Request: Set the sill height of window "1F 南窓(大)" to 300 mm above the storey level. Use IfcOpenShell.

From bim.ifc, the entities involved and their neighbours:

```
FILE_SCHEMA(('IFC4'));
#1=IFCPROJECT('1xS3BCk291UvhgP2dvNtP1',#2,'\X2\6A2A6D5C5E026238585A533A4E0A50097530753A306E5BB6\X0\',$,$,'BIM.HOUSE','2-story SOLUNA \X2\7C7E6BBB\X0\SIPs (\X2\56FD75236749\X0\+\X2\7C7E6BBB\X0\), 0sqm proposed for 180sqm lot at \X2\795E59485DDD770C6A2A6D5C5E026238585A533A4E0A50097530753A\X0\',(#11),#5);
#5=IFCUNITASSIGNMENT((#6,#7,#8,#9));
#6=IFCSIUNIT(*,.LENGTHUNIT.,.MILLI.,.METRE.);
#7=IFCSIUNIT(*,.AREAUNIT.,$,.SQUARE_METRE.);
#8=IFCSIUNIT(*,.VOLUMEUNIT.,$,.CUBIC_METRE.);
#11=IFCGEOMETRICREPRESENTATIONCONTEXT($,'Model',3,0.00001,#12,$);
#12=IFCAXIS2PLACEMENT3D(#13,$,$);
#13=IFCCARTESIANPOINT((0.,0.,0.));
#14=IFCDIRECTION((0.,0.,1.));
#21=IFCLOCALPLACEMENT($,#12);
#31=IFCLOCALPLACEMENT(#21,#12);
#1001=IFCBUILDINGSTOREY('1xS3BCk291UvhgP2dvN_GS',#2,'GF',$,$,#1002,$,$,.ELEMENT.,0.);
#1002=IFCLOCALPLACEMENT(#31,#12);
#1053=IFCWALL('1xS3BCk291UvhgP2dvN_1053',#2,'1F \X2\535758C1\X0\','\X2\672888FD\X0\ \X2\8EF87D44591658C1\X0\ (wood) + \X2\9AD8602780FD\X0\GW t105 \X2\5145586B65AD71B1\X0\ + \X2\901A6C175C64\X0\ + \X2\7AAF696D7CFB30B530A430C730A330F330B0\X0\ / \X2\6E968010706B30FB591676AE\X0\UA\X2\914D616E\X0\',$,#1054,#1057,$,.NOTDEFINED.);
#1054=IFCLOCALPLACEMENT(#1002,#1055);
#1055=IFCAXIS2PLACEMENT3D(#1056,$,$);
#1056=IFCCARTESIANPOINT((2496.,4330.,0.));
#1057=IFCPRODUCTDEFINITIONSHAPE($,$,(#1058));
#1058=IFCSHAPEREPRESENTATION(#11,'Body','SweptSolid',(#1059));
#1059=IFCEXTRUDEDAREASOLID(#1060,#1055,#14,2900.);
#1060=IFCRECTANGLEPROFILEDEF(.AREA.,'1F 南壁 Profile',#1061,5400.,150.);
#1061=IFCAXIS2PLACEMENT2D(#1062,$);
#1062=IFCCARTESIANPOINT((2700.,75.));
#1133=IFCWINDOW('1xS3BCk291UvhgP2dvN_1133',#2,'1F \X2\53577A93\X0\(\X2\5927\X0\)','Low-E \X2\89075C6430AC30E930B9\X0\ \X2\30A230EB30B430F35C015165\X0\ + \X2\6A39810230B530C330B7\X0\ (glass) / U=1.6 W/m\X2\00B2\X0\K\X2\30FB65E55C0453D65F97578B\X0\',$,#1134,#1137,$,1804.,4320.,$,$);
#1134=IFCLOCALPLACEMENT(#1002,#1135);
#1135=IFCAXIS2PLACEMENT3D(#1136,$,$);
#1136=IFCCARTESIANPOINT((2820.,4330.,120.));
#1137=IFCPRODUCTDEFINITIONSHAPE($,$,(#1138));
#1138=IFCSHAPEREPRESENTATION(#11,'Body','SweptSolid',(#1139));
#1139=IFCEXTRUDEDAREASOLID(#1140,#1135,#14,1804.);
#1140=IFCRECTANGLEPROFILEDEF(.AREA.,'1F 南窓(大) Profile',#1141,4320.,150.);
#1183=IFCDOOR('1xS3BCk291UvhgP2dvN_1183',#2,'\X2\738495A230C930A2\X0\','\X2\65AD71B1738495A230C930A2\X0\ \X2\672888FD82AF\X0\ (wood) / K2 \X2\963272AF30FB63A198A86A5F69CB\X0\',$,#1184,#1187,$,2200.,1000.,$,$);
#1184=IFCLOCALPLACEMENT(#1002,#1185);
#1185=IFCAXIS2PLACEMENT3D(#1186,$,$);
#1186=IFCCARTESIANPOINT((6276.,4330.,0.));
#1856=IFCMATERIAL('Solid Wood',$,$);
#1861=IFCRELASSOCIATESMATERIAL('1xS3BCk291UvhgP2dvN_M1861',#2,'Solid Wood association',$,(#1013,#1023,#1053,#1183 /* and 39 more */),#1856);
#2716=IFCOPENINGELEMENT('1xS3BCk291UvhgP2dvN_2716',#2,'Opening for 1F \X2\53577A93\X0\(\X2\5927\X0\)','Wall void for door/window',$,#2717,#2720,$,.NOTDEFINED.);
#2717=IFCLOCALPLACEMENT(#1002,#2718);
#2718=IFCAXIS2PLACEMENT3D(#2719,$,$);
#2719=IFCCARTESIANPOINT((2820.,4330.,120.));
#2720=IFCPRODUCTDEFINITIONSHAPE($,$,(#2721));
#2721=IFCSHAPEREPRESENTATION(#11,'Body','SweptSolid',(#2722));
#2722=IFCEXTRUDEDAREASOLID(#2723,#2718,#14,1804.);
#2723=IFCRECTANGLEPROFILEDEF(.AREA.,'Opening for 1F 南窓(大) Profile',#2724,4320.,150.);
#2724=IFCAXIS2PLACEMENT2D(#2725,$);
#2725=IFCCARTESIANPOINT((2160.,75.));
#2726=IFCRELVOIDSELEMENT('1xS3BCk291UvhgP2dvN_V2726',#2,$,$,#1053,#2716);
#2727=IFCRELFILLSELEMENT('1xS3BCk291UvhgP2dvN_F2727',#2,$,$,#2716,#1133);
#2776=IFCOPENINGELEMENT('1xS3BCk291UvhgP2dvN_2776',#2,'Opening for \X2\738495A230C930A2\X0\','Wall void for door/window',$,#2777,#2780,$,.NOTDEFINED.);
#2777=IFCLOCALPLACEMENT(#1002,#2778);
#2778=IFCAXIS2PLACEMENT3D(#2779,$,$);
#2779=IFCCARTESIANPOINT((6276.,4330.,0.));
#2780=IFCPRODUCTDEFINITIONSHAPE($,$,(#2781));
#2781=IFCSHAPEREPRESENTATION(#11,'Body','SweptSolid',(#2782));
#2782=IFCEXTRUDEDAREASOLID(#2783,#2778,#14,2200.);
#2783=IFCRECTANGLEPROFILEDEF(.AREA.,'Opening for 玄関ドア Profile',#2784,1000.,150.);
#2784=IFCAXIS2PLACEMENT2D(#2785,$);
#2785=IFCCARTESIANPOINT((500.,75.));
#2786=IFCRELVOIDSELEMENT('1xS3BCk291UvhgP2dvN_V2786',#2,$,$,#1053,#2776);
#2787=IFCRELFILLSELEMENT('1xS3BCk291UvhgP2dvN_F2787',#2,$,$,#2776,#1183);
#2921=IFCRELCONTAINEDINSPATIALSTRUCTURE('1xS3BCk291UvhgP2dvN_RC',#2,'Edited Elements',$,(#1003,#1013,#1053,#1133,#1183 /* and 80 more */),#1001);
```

```python
import numpy as np
import ifcopenshell
import ifcopenshell.api.geometry
import ifcopenshell.geom
import ifcopenshell.util.element
import ifcopenshell.util.placement
import ifcopenshell.util.shape
import ifcopenshell.util.unit

model = ifcopenshell.open("bim.ifc")
unit_scale = ifcopenshell.util.unit.calculate_unit_scale(model)

window = model.by_id(1133)
opening = window.FillsVoids[0].RelatingOpeningElement
storey = ifcopenshell.util.element.get_container(window, ifc_class="IfcBuildingStorey")
level = ifcopenshell.util.placement.get_local_placement(storey.ObjectPlacement)[2, 3]

# The opening's origin need not be at the sill, so measure its lowest point.
shape = ifcopenshell.geom.create_shape(ifcopenshell.geom.settings(), opening)
bottom = ifcopenshell.util.shape.get_shape_bottom_elevation(shape, shape.geometry) / unit_scale
dz = level + 0.3 / unit_scale - bottom

shift = np.array([0.0, 0.0, dz])
# The window is not placed relative to its opening, so move both.
for product in (opening, window):
    matrix = ifcopenshell.util.placement.get_local_placement(product.ObjectPlacement)
    matrix[:3, 3] += shift
    ifcopenshell.api.geometry.edit_object_placement(model, product=product, matrix=matrix, is_si=False)

print(f"moved by {dz * unit_scale:+.3f} m")

model.write("bim_updated.ifc")
```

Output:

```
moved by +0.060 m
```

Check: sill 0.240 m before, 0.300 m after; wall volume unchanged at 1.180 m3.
